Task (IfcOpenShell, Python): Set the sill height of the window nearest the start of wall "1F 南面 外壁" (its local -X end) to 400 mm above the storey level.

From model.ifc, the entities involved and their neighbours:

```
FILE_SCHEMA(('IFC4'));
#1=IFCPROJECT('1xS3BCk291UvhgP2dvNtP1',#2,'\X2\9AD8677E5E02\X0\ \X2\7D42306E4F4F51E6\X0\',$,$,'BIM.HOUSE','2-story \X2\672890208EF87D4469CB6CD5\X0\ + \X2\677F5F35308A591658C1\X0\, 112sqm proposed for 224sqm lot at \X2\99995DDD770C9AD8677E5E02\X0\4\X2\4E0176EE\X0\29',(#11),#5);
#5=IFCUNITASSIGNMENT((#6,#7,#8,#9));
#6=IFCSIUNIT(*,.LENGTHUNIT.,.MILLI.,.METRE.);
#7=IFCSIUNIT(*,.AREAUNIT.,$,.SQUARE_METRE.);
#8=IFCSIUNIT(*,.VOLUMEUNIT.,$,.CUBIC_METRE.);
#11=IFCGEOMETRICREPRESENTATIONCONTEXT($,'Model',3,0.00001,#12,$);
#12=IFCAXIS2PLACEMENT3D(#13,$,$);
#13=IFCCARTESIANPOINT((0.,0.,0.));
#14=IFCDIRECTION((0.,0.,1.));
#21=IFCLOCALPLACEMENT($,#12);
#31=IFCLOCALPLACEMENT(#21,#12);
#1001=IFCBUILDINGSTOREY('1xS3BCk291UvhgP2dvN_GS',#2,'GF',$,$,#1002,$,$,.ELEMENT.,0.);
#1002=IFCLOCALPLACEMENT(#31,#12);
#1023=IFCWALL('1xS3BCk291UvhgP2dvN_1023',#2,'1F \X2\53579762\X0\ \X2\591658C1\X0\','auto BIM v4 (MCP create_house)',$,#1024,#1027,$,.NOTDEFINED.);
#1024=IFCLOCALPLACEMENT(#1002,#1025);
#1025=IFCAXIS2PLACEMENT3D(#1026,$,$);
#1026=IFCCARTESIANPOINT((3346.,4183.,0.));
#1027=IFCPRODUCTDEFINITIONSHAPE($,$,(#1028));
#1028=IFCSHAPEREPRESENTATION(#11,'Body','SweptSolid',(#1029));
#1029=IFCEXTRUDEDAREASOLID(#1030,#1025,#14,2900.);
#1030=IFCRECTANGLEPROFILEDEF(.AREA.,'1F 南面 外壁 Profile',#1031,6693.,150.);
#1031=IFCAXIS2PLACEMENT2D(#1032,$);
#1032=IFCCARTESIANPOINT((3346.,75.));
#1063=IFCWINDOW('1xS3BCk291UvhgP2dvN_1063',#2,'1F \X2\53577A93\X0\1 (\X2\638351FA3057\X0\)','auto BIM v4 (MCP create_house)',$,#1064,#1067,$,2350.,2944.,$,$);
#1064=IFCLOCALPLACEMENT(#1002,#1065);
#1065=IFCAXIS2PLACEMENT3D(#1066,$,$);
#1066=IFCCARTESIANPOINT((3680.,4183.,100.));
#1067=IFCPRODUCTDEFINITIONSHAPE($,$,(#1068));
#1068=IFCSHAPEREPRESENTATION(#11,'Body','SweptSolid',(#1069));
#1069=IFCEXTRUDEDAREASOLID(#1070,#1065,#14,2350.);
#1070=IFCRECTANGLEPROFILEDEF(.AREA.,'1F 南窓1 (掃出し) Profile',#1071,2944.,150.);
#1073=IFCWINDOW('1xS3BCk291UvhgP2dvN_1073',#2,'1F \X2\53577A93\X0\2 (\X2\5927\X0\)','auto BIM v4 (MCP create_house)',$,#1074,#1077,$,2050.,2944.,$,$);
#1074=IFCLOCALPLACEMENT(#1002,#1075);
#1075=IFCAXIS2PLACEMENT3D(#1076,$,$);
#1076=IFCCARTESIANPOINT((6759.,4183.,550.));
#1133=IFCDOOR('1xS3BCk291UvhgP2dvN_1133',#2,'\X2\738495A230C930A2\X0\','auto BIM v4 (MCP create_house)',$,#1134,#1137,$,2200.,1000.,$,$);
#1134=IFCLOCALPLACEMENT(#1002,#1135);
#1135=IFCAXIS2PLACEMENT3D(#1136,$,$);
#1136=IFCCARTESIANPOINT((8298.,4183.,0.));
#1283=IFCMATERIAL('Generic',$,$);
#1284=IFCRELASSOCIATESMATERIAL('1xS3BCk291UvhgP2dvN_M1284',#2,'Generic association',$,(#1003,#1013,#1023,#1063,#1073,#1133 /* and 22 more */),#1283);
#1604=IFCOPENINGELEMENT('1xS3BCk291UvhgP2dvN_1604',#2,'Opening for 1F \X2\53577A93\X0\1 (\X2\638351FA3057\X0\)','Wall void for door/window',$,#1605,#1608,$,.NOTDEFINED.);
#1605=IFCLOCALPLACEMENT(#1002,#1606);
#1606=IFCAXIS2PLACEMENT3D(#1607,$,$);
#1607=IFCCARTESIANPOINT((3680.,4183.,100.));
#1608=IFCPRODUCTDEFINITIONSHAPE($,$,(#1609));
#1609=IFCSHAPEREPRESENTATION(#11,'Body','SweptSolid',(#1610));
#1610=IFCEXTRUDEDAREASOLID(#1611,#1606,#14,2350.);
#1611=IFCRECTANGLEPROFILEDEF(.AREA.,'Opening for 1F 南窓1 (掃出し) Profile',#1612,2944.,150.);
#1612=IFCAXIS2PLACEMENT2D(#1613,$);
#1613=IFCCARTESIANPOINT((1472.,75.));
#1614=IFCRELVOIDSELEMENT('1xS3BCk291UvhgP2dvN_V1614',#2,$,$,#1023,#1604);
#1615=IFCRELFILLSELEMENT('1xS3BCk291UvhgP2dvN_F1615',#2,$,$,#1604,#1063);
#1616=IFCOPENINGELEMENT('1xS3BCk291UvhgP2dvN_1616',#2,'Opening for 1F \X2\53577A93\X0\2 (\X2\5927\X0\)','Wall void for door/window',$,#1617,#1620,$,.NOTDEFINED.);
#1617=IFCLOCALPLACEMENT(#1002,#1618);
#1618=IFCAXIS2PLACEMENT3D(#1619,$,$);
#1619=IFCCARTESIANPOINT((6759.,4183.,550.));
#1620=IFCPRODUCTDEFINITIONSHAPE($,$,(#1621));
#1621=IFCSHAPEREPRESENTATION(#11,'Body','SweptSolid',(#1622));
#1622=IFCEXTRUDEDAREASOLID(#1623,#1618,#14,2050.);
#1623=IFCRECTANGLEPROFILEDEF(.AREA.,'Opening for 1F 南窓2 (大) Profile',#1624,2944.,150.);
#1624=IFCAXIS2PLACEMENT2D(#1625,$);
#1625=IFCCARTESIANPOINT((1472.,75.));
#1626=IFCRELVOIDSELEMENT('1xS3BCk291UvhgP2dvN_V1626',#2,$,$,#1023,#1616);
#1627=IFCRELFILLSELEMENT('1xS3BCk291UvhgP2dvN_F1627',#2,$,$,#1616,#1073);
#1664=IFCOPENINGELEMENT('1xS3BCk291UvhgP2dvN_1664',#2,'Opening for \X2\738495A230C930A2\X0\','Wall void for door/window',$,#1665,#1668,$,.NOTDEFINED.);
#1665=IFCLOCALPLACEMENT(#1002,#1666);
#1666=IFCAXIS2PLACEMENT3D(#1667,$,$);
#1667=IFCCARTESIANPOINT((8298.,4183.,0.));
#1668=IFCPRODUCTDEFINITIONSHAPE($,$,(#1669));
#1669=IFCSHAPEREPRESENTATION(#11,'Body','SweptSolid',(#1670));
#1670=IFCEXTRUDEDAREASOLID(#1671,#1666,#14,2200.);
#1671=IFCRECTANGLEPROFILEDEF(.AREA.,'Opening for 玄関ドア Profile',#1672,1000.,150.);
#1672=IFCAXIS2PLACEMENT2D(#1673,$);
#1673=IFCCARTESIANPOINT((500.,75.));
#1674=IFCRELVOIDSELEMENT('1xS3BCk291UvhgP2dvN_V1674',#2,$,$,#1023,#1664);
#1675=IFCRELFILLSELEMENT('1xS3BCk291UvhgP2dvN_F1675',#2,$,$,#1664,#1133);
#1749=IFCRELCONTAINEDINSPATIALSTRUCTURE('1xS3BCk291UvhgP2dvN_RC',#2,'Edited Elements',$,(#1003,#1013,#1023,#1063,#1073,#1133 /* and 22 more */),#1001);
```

```python
import numpy as np
import ifcopenshell
import ifcopenshell.api.geometry
import ifcopenshell.geom
import ifcopenshell.util.element
import ifcopenshell.util.placement
import ifcopenshell.util.shape
import ifcopenshell.util.unit

model = ifcopenshell.open("model.ifc")
unit_scale = ifcopenshell.util.unit.calculate_unit_scale(model)

window = model.by_id(1063)
opening = window.FillsVoids[0].RelatingOpeningElement
storey = ifcopenshell.util.element.get_container(window, ifc_class="IfcBuildingStorey")
level = ifcopenshell.util.placement.get_local_placement(storey.ObjectPlacement)[2, 3]

# The opening's origin need not be at the sill, so measure its lowest point.
shape = ifcopenshell.geom.create_shape(ifcopenshell.geom.settings(), opening)
bottom = ifcopenshell.util.shape.get_shape_bottom_elevation(shape, shape.geometry) / unit_scale
dz = level + 400.0 - bottom

shift = np.array([0.0, 0.0, dz])
# The window is not placed relative to its opening, so move both.
for product in (opening, window):
    matrix = ifcopenshell.util.placement.get_local_placement(product.ObjectPlacement)
    matrix[:3, 3] += shift
    ifcopenshell.api.geometry.edit_object_placement(model, product=product, matrix=matrix, is_si=False)

print(f"moved by {dz * unit_scale:+.3f} m")

model.write("model_v2.ifc")
```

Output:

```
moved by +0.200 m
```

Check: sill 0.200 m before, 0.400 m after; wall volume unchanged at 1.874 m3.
